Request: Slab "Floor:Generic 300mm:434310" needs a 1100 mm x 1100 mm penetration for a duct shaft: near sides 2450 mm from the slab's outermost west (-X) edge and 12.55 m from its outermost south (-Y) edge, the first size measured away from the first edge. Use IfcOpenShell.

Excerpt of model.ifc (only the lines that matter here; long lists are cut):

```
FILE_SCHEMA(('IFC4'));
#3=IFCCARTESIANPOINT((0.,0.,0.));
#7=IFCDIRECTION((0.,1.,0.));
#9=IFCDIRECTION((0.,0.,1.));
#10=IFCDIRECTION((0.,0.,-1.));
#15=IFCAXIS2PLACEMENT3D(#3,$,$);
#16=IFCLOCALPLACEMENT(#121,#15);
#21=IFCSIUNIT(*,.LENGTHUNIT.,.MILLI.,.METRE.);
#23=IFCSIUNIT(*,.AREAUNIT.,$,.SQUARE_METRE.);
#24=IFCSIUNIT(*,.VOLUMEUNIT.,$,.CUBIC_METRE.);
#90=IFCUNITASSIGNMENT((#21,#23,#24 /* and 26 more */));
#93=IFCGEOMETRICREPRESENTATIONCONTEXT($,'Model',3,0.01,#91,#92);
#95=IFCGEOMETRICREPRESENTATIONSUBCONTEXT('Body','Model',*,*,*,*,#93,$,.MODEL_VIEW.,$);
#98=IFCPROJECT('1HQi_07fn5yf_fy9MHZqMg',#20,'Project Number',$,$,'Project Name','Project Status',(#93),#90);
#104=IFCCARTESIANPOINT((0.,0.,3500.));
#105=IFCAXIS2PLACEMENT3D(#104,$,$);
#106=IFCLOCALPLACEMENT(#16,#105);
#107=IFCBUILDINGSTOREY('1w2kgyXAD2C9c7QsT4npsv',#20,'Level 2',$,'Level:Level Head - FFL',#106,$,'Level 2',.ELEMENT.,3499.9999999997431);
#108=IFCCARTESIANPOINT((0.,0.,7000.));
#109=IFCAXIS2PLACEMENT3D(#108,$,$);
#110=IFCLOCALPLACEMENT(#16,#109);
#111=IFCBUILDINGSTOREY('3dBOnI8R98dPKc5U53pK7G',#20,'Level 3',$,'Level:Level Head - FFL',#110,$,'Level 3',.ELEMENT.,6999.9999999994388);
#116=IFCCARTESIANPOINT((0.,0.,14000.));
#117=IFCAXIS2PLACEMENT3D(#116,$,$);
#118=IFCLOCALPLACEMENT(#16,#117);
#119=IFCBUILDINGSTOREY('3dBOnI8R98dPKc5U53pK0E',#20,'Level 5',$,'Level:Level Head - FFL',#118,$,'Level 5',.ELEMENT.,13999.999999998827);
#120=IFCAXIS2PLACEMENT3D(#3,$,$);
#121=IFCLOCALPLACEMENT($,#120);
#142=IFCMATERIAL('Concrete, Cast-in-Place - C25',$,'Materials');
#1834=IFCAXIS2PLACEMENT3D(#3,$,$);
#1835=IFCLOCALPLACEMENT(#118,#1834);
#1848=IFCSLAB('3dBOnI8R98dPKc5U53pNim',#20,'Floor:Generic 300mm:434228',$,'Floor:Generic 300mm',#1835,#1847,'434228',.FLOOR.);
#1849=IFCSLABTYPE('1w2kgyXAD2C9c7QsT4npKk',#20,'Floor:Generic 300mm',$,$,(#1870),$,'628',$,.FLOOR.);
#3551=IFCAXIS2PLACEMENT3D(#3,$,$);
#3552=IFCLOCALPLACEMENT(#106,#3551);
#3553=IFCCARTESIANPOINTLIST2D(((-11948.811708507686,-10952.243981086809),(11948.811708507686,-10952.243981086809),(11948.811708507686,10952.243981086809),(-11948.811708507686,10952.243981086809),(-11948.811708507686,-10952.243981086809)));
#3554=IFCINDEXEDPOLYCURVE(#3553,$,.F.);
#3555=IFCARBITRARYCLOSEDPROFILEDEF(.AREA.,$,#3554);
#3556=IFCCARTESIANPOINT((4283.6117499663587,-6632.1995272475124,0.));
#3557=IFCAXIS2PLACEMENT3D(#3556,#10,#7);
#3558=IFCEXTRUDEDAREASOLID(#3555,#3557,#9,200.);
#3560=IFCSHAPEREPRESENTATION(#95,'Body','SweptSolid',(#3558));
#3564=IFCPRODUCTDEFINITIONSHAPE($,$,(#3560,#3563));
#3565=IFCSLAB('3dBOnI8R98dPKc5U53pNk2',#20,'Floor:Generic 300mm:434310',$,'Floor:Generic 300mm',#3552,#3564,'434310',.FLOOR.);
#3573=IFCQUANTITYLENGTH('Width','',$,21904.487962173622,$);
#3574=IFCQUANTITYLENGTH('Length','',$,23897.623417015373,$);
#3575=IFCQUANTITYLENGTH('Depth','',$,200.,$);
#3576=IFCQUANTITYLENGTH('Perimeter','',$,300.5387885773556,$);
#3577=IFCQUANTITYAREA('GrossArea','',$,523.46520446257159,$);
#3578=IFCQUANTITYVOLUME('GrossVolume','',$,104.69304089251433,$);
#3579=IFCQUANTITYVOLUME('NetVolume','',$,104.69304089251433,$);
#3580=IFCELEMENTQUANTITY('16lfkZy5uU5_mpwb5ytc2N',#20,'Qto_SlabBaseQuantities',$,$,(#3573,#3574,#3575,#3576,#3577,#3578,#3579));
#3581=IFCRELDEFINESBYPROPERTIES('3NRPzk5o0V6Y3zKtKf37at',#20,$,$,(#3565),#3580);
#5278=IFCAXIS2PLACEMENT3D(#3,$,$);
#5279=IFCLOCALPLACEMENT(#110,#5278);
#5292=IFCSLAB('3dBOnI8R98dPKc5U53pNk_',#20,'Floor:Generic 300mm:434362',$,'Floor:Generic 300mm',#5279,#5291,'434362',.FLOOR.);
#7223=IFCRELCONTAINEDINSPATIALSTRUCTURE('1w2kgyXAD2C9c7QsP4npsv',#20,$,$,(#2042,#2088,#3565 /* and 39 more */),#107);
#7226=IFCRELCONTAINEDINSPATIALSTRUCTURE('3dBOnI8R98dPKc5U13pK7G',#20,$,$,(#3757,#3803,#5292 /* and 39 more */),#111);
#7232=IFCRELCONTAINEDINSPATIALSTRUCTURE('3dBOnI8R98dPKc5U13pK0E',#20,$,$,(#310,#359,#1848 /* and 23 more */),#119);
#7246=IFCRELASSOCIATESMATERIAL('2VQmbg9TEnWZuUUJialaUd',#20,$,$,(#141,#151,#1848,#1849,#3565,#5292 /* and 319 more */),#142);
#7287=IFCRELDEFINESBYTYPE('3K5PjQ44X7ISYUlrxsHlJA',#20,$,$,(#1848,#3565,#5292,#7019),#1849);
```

```python
import numpy as np
import ifcopenshell
import ifcopenshell.api.feature
import ifcopenshell.api.geometry
import ifcopenshell.api.pset
import ifcopenshell.api.root
import ifcopenshell.geom
import ifcopenshell.util.element
import ifcopenshell.util.placement
import ifcopenshell.util.representation
import ifcopenshell.util.shape
import ifcopenshell.util.unit

model = ifcopenshell.open("model.ifc")
unit_scale = ifcopenshell.util.unit.calculate_unit_scale(model)
volume_scale = ifcopenshell.util.unit.calculate_unit_scale(model, "VOLUMEUNIT")
settings = ifcopenshell.geom.settings()


def volume(element):
    """Net volume in cubic metres, openings subtracted."""
    shape = ifcopenshell.geom.create_shape(settings, element)
    return ifcopenshell.util.shape.get_volume(shape.geometry)


slab = model.by_guid("3dBOnI8R98dPKc5U53pNk2")
before = volume(slab)

# Extent in the slab's own axes, in metres. The edges named are its -X and -Y sides.
slab_shape = ifcopenshell.geom.create_shape(settings, slab)
vertices = ifcopenshell.util.shape.get_vertices(slab_shape.geometry)
x_min, y_min, bottom = vertices.min(axis=0)
top = vertices[:, 2].max()

opening = ifcopenshell.api.root.create_entity(model, ifc_class="IfcOpeningElement", name="Duct shaft opening", predefined_type="OPENING")
context = ifcopenshell.util.representation.get_context(model, "Model", "Body", "MODEL_VIEW")
width, depth = 1.1, 1.1
outline = [(0.0, 0.0), (width, 0.0), (width, depth), (0.0, depth), (0.0, 0.0)]
# Overshoot both faces by 50 mm so the cut is clean.
shape = ifcopenshell.api.geometry.add_slab_representation(
    model, context=context, depth=top - bottom + 0.1, polyline=outline
)
ifcopenshell.api.geometry.assign_representation(model, product=opening, representation=shape)

matrix = ifcopenshell.util.placement.get_local_placement(slab.ObjectPlacement)
matrix[:, 3] = matrix @ np.append(np.array([x_min + 2.45, y_min + 12.55, bottom - 0.05]) / unit_scale, 1.0)
ifcopenshell.api.geometry.edit_object_placement(model, product=opening, matrix=matrix, is_si=False)
ifcopenshell.api.feature.add_feature(model, feature=opening, element=slab)

after = volume(slab)

# Update the slab's stored quantities.
qto = model.by_id(ifcopenshell.util.element.get_pset(slab, "Qto_SlabBaseQuantities", should_inherit=False)["id"])
ifcopenshell.api.pset.edit_qto(model, qto=qto, properties={"NetVolume": after / volume_scale})

print(f"slab volume {before:.3f} -> {after:.3f} m3")

model.write("model_updated.ifc")
```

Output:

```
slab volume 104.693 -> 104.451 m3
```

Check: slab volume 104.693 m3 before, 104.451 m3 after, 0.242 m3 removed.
